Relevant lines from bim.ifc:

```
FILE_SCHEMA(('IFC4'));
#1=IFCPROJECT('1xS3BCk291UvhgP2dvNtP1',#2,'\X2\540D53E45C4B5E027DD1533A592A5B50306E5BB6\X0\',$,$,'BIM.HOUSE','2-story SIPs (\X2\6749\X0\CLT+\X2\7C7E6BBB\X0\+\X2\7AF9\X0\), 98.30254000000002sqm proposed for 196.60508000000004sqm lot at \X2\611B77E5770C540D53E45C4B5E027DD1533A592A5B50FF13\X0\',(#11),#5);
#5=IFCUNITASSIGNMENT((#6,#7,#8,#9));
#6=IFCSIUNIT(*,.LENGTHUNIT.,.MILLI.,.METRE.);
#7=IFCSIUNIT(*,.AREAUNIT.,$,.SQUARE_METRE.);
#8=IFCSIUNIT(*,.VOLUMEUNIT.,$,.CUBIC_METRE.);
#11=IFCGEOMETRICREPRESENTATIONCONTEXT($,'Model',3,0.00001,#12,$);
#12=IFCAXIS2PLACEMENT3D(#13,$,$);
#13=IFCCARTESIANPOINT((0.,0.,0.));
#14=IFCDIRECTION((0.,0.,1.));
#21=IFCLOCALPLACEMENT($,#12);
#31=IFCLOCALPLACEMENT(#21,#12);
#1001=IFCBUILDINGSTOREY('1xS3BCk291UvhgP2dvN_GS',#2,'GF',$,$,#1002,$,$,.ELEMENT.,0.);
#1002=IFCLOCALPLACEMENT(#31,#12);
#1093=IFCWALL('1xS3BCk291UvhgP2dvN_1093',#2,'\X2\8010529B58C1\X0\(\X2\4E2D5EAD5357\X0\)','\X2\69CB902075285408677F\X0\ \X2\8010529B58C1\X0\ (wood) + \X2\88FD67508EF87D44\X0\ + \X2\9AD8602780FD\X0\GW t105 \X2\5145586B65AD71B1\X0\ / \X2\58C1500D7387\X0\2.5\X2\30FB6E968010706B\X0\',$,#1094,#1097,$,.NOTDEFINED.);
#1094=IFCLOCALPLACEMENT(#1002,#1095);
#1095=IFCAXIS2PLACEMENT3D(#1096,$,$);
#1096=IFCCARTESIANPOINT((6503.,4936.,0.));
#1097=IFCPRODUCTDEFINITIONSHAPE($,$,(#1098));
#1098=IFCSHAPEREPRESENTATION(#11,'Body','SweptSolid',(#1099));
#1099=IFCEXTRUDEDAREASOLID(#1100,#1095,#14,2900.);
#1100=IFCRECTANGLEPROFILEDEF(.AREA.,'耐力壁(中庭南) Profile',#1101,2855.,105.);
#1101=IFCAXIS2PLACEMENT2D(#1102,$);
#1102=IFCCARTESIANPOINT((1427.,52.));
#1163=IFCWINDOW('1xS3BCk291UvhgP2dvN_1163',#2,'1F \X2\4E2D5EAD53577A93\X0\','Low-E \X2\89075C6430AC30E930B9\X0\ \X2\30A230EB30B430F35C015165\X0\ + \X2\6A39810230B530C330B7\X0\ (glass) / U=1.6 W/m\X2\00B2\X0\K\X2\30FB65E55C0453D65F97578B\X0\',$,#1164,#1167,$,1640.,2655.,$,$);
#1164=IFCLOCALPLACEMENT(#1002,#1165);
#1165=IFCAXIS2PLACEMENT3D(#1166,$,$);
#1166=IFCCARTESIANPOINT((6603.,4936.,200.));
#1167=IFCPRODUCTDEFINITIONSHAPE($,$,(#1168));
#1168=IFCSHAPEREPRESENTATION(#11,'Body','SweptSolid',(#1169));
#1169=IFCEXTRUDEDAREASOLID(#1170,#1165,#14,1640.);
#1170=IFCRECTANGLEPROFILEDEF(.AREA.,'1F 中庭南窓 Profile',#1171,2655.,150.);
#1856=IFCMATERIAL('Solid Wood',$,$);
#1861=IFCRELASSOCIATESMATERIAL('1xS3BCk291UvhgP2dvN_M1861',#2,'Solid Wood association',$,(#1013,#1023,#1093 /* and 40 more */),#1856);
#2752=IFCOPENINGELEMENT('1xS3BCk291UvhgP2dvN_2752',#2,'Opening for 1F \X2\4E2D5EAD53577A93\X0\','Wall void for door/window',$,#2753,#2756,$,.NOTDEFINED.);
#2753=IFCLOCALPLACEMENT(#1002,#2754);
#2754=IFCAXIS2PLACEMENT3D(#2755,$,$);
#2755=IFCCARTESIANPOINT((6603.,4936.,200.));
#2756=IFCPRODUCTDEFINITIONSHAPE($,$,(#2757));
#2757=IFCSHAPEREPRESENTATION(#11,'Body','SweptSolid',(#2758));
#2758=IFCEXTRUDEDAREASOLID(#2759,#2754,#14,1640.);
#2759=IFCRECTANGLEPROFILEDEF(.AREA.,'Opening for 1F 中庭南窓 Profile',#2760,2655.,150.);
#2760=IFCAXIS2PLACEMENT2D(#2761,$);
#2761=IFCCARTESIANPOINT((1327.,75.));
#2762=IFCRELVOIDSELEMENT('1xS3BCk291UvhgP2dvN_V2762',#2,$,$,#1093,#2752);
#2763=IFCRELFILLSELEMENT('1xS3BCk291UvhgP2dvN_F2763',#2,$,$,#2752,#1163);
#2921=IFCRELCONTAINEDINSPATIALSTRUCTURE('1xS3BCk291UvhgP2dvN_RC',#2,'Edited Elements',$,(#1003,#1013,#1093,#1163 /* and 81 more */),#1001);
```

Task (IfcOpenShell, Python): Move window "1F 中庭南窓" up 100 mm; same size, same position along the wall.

```python
import numpy as np
import ifcopenshell
import ifcopenshell.api.geometry
import ifcopenshell.util.placement
import ifcopenshell.util.unit

model = ifcopenshell.open("bim.ifc")
unit_scale = ifcopenshell.util.unit.calculate_unit_scale(model)

window = model.by_guid("1xS3BCk291UvhgP2dvN_1163")
opening = window.FillsVoids[0].RelatingOpeningElement
dz = 0.1 / unit_scale

shift = np.array([0.0, 0.0, dz])
# The window is not placed relative to its opening, so move both.
for product in (opening, window):
    matrix = ifcopenshell.util.placement.get_local_placement(product.ObjectPlacement)
    matrix[:3, 3] += shift
    ifcopenshell.api.geometry.edit_object_placement(model, product=product, matrix=matrix, is_si=False)

print(f"moved by {dz * unit_scale:+.3f} m")

model.write("bim_updated.ifc")
```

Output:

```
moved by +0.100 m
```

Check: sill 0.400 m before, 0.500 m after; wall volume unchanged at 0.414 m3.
